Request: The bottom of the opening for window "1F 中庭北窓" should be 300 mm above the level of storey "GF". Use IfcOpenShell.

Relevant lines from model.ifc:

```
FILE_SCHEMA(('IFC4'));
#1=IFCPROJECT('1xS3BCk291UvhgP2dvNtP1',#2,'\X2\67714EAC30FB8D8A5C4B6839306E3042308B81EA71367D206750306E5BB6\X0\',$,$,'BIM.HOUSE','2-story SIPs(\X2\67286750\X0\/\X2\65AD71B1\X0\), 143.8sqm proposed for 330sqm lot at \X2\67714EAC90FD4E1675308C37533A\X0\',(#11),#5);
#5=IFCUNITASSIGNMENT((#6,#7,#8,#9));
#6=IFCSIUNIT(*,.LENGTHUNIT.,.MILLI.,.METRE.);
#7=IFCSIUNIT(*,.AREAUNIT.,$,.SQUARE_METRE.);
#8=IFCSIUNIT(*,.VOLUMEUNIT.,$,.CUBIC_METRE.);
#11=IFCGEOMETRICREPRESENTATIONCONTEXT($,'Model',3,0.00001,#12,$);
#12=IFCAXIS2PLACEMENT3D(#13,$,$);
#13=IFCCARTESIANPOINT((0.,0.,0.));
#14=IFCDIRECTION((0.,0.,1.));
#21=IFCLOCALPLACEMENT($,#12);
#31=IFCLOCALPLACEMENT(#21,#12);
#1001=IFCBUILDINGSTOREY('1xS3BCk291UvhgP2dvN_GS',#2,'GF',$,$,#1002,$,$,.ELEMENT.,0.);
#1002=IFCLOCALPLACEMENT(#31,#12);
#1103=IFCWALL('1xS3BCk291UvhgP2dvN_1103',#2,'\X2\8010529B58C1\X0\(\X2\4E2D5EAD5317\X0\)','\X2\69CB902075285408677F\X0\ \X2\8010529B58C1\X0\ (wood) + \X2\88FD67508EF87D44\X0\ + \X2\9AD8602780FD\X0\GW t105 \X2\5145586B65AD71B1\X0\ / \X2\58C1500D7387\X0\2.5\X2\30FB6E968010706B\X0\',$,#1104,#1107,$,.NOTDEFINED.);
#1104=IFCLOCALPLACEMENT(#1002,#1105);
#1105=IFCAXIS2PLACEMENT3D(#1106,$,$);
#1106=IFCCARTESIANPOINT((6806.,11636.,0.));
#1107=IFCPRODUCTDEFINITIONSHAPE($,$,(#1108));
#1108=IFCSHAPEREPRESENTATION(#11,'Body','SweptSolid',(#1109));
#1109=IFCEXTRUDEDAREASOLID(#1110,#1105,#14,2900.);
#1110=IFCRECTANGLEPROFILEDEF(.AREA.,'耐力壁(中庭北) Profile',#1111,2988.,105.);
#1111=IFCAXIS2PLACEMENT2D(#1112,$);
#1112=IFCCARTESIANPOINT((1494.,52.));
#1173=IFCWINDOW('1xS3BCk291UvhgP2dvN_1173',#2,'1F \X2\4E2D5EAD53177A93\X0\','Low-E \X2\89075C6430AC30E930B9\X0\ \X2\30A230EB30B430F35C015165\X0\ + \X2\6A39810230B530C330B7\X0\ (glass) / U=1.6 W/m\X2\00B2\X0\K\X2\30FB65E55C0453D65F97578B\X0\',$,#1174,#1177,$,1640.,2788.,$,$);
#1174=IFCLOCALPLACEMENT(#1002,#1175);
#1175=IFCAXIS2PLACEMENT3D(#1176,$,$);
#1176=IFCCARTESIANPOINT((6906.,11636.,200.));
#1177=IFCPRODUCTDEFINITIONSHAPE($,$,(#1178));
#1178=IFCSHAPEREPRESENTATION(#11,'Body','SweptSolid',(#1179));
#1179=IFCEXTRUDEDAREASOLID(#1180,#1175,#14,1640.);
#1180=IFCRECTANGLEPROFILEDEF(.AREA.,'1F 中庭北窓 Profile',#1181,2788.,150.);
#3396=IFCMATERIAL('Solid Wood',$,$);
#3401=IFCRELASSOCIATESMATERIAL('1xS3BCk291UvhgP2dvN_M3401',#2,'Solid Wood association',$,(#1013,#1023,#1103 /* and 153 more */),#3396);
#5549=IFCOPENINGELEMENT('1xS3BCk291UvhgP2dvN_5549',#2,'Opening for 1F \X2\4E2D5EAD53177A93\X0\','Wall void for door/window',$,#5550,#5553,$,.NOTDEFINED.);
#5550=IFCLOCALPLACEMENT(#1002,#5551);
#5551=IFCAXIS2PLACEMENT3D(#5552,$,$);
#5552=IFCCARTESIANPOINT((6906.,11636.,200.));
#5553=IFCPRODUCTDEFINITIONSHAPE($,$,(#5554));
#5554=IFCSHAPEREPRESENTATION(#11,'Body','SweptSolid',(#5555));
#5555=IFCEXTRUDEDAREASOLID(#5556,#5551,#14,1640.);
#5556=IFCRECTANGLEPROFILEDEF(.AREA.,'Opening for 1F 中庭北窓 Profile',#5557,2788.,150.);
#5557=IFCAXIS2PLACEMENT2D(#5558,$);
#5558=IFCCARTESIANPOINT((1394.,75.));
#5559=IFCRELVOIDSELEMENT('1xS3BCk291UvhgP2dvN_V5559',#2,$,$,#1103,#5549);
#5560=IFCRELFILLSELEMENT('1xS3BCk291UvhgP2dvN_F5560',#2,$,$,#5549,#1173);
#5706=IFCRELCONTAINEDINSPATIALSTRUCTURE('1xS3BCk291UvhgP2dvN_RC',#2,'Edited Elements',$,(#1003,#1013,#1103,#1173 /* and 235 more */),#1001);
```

```python
import numpy as np
import ifcopenshell
import ifcopenshell.api.geometry
import ifcopenshell.geom
import ifcopenshell.util.element
import ifcopenshell.util.placement
import ifcopenshell.util.shape
import ifcopenshell.util.unit

model = ifcopenshell.open("model.ifc")
unit_scale = ifcopenshell.util.unit.calculate_unit_scale(model)

window = model.by_guid("1xS3BCk291UvhgP2dvN_1173")
opening = window.FillsVoids[0].RelatingOpeningElement
storey = ifcopenshell.util.element.get_container(window, ifc_class="IfcBuildingStorey")
level = ifcopenshell.util.placement.get_local_placement(storey.ObjectPlacement)[2, 3]

# The opening's origin need not be at the sill, so measure its lowest point.
shape = ifcopenshell.geom.create_shape(ifcopenshell.geom.settings(), opening)
bottom = ifcopenshell.util.shape.get_shape_bottom_elevation(shape, shape.geometry) / unit_scale
dz = level + 300.0 - bottom

shift = np.array([0.0, 0.0, dz])
# The window is not placed relative to its opening, so move both.
for product in (opening, window):
    matrix = ifcopenshell.util.placement.get_local_placement(product.ObjectPlacement)
    matrix[:3, 3] += shift
    ifcopenshell.api.geometry.edit_object_placement(model, product=product, matrix=matrix, is_si=False)

print(f"moved by {dz * unit_scale:+.3f} m")

model.write("model_rev.ifc")
```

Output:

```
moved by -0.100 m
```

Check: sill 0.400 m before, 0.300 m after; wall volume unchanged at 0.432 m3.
